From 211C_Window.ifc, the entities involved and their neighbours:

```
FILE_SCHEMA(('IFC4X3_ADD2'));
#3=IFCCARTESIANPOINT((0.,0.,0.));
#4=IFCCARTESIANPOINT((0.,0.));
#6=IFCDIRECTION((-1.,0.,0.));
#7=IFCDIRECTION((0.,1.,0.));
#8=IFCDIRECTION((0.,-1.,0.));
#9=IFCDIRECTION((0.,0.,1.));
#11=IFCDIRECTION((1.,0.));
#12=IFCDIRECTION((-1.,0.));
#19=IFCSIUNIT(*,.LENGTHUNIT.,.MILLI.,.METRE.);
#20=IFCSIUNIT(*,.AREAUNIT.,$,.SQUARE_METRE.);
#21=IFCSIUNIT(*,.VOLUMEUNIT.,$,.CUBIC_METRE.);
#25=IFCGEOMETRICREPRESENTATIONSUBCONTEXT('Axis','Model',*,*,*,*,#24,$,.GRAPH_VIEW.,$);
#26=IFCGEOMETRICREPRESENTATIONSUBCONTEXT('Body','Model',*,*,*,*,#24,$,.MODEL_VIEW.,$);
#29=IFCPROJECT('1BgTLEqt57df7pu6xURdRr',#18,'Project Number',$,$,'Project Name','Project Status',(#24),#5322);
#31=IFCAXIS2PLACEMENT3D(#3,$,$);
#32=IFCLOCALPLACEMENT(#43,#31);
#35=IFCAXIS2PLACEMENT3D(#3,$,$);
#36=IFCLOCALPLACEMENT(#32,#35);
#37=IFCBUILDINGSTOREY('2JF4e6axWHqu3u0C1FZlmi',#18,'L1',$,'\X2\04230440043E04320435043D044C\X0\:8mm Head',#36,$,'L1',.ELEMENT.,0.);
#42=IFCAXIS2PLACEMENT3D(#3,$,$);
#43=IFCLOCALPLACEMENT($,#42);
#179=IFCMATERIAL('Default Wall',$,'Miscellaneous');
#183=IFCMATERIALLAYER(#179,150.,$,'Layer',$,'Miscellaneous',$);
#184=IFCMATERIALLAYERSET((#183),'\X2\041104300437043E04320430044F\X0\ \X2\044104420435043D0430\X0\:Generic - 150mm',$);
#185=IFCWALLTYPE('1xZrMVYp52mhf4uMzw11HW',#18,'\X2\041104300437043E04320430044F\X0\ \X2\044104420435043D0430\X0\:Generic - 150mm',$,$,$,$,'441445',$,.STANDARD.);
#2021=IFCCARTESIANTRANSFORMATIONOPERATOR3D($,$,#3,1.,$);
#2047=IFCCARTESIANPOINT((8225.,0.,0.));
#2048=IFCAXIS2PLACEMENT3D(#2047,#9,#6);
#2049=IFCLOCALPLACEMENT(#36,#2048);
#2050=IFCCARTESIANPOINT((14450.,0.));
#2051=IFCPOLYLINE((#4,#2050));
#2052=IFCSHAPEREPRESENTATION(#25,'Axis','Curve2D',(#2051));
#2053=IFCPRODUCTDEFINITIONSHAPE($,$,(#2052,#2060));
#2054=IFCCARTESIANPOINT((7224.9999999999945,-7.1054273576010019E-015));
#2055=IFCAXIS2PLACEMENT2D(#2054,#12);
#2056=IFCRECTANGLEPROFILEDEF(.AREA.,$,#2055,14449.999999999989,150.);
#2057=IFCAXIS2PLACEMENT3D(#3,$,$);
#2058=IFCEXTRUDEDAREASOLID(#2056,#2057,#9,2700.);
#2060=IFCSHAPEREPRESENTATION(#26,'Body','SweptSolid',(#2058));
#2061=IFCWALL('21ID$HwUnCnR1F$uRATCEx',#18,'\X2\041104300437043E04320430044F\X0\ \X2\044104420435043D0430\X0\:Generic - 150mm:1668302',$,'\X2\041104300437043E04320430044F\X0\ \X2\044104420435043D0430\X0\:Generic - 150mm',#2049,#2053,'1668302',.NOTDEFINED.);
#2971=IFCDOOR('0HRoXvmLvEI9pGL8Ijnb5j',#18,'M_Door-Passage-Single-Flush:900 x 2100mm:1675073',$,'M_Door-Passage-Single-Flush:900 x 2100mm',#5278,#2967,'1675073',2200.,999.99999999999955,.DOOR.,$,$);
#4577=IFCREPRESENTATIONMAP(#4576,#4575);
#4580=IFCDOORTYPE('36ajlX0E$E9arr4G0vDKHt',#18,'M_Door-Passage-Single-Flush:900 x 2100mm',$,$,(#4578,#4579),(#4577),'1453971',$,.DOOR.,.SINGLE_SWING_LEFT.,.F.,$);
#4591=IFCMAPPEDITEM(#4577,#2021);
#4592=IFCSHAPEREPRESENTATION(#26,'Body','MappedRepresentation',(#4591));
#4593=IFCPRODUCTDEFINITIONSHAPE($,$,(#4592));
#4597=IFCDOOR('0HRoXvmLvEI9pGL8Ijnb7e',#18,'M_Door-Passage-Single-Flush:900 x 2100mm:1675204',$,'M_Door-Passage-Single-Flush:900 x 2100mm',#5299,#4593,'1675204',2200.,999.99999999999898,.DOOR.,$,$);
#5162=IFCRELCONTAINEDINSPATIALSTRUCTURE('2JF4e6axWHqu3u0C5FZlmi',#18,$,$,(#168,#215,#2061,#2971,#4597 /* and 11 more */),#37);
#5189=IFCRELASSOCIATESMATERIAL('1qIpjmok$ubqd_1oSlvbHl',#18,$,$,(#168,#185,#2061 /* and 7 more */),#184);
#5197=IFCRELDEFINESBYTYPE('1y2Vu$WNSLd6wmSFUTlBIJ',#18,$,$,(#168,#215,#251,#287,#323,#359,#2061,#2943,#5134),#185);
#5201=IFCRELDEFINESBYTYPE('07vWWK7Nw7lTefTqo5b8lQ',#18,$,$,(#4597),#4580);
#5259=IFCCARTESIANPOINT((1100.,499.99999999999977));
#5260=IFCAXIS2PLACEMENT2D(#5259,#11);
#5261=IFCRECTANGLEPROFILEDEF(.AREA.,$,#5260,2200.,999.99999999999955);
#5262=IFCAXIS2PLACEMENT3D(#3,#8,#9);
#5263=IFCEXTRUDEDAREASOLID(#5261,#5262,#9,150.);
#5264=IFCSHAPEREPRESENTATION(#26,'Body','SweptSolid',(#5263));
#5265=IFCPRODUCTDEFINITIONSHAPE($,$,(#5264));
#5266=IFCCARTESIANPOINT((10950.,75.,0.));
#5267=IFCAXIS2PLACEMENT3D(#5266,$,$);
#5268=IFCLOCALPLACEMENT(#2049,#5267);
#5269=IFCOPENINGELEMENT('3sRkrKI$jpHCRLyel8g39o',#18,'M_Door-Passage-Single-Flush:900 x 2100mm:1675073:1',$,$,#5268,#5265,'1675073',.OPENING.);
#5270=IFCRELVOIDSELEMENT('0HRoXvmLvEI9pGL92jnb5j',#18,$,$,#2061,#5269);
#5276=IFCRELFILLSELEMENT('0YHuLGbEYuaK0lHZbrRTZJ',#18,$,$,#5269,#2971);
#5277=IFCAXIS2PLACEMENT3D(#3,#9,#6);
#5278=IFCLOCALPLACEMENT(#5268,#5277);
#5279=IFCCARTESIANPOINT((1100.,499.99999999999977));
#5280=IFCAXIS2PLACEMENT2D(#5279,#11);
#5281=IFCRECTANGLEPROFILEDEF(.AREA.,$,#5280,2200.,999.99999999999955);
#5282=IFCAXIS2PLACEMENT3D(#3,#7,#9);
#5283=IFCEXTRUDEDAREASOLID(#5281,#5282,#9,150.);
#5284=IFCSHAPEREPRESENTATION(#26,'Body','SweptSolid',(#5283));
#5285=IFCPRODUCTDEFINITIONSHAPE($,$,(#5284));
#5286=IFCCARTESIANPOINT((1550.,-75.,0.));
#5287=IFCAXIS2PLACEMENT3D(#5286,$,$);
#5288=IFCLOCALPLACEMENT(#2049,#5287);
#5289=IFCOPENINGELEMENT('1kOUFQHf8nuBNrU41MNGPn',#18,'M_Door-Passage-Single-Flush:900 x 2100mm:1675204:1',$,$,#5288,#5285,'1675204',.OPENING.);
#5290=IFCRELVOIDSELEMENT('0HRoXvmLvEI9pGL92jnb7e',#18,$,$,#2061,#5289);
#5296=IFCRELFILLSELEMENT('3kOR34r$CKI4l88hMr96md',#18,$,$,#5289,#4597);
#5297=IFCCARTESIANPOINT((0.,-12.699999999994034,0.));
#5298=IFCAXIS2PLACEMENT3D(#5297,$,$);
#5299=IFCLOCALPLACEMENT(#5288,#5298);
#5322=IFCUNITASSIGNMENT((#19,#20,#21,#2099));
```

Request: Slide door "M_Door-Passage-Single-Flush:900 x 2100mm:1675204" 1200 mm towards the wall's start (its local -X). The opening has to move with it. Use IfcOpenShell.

```python
import ifcopenshell
import ifcopenshell.api.geometry
import ifcopenshell.util.placement
import ifcopenshell.util.unit

model = ifcopenshell.open("211C_Window.ifc")
unit_scale = ifcopenshell.util.unit.calculate_unit_scale(model)

door = model.by_guid("0HRoXvmLvEI9pGL8Ijnb7e")
opening = door.FillsVoids[0].RelatingOpeningElement
wall = opening.VoidsElements[0].RelatingBuildingElement

wall_matrix = ifcopenshell.util.placement.get_local_placement(wall.ObjectPlacement)
shift = wall_matrix[:3, 0] * -1.2 / unit_scale
before = ifcopenshell.util.placement.get_local_placement(door.ObjectPlacement)[:3, 3].copy()

# The door is placed relative to its opening, so it follows when the opening moves.
matrix = ifcopenshell.util.placement.get_local_placement(opening.ObjectPlacement)
matrix[:3, 3] += shift
ifcopenshell.api.geometry.edit_object_placement(
    model, product=opening, matrix=matrix, is_si=False, should_transform_children=True
)

after = ifcopenshell.util.placement.get_local_placement(door.ObjectPlacement)[:3, 3]
print("door moved by", (after - before).round(3) + 0.0)

model.write("211C_Window-out.ifc")
```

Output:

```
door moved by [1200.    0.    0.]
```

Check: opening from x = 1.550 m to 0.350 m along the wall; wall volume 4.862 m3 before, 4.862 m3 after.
